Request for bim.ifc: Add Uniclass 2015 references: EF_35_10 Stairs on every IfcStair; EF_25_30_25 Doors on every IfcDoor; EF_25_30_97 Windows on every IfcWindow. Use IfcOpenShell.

First a look at what the model holds.

```python
import ifcopenshell

model = ifcopenshell.open("bim.ifc")
print(model.schema)
print("classifications:", [c.Name for c in model.by_type("IfcClassification")])
for ifc_class in ("IfcDoor", "IfcRoof", "IfcStair", "IfcWall", "IfcWindow"):
    print(ifc_class, len(model.by_type(ifc_class)))
```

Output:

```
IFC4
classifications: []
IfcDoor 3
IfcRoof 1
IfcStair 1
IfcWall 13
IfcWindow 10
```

```python
import ifcopenshell
import ifcopenshell.api.classification

model = ifcopenshell.open("bim.ifc")

system = ifcopenshell.api.classification.add_classification(model, classification="Uniclass 2015")

codes = {
    "IfcStair": ("EF_35_10", "Stairs"),
    "IfcDoor": ("EF_25_30_25", "Doors"),
    "IfcWindow": ("EF_25_30_97", "Windows"),
}
for ifc_class, (code, name) in codes.items():
    products = model.by_type(ifc_class)
    ifcopenshell.api.classification.add_reference(
        model, products=products, classification=system, identification=code, name=name
    )
    print(code, len(products))

model.write("bim_edited.ifc")
```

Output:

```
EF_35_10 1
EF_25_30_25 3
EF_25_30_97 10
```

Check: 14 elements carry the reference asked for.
